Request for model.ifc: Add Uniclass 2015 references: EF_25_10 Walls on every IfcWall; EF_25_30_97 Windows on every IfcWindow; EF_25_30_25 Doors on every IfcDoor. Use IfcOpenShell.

First a look at what the model holds.

```python
import ifcopenshell

model = ifcopenshell.open("model.ifc")
print(model.schema)
print("classifications:", [c.Name for c in model.by_type("IfcClassification")])
for ifc_class in ("IfcDoor", "IfcRoof", "IfcStair", "IfcWall", "IfcWindow"):
    print(ifc_class, len(model.by_type(ifc_class)))
```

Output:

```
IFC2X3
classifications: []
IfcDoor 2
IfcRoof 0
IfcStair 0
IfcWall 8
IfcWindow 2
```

```python
import ifcopenshell
import ifcopenshell.api.classification

model = ifcopenshell.open("model.ifc")

# IFC2X3 requires Source and Edition and has no link from the project to the system.
system = model.create_entity("IfcClassification", Source="NBS", Edition="2015", Name="Uniclass 2015")

codes = {
    "IfcWall": ("EF_25_10", "Walls"),
    "IfcWindow": ("EF_25_30_97", "Windows"),
    "IfcDoor": ("EF_25_30_25", "Doors"),
}
for ifc_class, (code, name) in codes.items():
    products = model.by_type(ifc_class)
    ifcopenshell.api.classification.add_reference(
        model, products=products, classification=system, identification=code, name=name
    )
    print(code, len(products))

model.write("model_v2.ifc")
```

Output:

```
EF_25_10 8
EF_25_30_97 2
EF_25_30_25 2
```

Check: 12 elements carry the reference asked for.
